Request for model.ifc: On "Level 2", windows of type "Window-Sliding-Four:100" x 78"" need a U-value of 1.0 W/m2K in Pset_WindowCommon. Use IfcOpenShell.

First a look at what the model holds.

```python
import ifcopenshell
import ifcopenshell.util.element

model = ifcopenshell.open("model.ifc")
print(model.schema)
storey = next(s for s in model.by_type("IfcBuildingStorey") if s.Name == "Level 2")
windows = [e for e in ifcopenshell.util.element.get_decomposition(storey) if e.is_a("IfcWindow")]
seen = {}
for e in windows:
    element_type = ifcopenshell.util.element.get_type(e)
    key = (element_type.Name if element_type != e and element_type else None, ifcopenshell.util.element.get_pset(e, "Pset_WindowCommon", "ThermalTransmittance"))
    seen[key] = seen.get(key, 0) + 1
for (name, value), count in sorted(seen.items(), key=str):
    print(count, "x", name, "|", value)
```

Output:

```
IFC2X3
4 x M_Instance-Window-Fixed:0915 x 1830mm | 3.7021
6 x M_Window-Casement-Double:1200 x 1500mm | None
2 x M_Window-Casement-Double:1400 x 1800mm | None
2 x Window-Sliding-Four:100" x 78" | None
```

```python
import ifcopenshell
import ifcopenshell.api.pset
import ifcopenshell.util.element

model = ifcopenshell.open("model.ifc")

storey = next(s for s in model.by_type("IfcBuildingStorey") if s.Name == "Level 2")
windows = [e for e in ifcopenshell.util.element.get_decomposition(storey) if e.is_a("IfcWindow")]

count = 0
for e in windows:
    element_type = ifcopenshell.util.element.get_type(e)
    if element_type in (None, e) or element_type.Name != 'Window-Sliding-Four:100" x 78"':
        continue
    # add_pset returns the element's existing set when there is one.
    pset = ifcopenshell.api.pset.add_pset(model, product=e, name="Pset_WindowCommon")
    ifcopenshell.api.pset.edit_pset(model, pset=pset, properties={"ThermalTransmittance": 1.0})
    count += 1

print(count, "windows updated")

model.write("model_rev.ifc")
```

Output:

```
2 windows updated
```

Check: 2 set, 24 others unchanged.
